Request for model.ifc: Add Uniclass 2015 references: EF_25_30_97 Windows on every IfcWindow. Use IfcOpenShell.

First a look at what the model holds.

```python
import ifcopenshell

model = ifcopenshell.open("model.ifc")
print(model.schema)
print("classifications:", [c.Name for c in model.by_type("IfcClassification")])
for ifc_class in ("IfcDoor", "IfcRoof", "IfcStair", "IfcWall", "IfcWindow"):
    print(ifc_class, len(model.by_type(ifc_class)))
```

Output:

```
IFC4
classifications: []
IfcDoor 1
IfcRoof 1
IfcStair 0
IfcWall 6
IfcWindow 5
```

```python
import ifcopenshell
import ifcopenshell.api.classification

model = ifcopenshell.open("model.ifc")

system = ifcopenshell.api.classification.add_classification(model, classification="Uniclass 2015")

codes = {
    "IfcWindow": ("EF_25_30_97", "Windows"),
}
for ifc_class, (code, name) in codes.items():
    products = model.by_type(ifc_class)
    ifcopenshell.api.classification.add_reference(
        model, products=products, classification=system, identification=code, name=name
    )
    print(code, len(products))

model.write("model_v2.ifc")
```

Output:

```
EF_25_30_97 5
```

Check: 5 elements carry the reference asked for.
